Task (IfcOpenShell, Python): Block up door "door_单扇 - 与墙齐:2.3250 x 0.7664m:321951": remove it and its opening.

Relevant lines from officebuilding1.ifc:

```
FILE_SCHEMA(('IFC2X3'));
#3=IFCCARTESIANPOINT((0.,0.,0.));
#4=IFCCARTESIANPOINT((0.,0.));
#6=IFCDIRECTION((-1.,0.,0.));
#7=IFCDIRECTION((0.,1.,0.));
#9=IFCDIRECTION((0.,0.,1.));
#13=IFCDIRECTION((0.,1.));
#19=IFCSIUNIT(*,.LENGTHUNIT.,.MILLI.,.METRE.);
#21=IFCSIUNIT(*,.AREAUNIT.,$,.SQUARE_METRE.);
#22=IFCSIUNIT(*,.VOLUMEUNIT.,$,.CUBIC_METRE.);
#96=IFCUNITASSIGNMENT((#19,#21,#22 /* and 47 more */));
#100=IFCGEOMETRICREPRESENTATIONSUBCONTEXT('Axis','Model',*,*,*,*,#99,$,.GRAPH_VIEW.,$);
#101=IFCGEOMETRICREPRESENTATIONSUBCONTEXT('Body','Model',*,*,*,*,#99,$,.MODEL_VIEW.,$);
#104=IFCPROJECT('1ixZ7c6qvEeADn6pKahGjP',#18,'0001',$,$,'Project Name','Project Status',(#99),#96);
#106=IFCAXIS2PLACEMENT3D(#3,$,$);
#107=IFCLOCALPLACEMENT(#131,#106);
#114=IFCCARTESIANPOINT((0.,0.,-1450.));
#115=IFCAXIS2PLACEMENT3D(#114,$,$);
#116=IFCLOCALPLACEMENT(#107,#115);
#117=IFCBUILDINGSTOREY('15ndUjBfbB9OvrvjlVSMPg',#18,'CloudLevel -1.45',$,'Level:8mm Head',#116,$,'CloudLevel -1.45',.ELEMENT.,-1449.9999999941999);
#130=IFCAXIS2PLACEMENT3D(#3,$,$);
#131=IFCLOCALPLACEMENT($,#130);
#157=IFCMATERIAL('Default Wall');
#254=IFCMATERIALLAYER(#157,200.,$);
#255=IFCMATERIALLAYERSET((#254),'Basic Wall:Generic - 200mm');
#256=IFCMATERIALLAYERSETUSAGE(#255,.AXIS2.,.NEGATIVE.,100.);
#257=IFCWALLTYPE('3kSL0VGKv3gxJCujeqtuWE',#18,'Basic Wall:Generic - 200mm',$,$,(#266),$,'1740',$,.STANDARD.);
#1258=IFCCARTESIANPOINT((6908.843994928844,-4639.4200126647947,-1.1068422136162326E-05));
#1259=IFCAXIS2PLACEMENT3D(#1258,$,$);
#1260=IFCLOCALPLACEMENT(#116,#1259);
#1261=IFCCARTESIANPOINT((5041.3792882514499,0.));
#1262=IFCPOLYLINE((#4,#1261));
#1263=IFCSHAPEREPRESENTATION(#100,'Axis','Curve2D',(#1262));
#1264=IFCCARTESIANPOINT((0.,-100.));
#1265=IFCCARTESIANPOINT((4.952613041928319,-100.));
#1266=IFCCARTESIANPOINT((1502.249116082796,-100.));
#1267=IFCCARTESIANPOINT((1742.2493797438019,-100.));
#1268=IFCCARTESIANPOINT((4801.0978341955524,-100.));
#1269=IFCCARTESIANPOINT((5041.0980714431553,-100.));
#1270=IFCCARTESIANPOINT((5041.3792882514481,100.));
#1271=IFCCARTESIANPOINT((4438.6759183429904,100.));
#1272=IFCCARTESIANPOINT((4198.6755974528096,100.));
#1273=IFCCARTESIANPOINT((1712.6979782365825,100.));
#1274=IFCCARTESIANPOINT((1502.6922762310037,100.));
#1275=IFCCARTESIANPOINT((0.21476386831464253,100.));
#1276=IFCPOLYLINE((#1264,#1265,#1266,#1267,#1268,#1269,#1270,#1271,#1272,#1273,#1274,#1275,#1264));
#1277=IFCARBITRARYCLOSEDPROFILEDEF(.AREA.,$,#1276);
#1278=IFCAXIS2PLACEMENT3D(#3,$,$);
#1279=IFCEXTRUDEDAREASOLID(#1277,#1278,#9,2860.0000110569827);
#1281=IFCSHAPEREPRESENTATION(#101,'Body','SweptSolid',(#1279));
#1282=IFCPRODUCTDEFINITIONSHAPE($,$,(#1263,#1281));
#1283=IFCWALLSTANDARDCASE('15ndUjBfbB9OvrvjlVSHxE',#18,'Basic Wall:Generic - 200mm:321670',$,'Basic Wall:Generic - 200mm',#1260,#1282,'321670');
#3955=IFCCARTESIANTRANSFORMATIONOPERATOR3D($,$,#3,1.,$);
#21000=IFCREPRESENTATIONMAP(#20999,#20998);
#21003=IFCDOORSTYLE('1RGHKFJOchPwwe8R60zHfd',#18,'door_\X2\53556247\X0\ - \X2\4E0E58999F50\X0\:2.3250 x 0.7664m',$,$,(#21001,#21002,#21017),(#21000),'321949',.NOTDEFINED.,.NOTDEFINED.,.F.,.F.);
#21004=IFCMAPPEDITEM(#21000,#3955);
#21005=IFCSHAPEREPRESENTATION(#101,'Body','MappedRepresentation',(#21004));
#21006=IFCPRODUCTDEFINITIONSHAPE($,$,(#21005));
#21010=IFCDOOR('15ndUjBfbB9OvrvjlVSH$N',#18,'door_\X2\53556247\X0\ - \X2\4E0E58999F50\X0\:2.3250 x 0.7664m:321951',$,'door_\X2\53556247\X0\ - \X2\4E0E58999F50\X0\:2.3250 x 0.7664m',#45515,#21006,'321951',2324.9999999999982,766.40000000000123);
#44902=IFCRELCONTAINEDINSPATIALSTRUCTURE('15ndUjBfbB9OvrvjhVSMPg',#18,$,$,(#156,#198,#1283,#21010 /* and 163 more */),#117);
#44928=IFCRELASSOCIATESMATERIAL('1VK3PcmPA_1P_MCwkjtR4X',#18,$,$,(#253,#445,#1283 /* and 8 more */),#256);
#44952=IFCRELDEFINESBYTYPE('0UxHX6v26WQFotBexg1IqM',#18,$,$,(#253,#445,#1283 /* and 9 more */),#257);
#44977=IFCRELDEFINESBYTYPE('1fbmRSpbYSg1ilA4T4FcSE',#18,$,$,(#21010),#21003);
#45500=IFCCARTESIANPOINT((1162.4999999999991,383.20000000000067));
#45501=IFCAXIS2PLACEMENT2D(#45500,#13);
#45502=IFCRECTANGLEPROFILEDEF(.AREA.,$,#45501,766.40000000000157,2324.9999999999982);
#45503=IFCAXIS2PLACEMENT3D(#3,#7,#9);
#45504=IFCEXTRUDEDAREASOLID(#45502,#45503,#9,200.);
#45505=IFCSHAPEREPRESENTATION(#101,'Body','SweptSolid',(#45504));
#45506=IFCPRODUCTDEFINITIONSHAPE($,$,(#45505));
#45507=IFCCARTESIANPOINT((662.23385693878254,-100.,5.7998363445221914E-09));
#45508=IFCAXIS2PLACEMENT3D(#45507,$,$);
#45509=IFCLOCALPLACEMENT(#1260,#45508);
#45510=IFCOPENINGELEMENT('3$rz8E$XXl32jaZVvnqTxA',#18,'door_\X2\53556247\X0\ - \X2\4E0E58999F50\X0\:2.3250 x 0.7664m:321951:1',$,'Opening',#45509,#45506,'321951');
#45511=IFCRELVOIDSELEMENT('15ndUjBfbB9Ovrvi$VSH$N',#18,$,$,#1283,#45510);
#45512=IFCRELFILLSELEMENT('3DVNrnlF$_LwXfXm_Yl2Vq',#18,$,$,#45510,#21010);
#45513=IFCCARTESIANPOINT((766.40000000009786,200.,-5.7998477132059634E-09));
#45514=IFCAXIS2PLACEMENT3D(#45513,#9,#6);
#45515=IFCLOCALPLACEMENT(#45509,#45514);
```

```python
import ifcopenshell
import ifcopenshell.api.feature
import ifcopenshell.api.root
import ifcopenshell.geom
import ifcopenshell.util.shape

model = ifcopenshell.open("officebuilding1.ifc")
settings = ifcopenshell.geom.settings()


def volume(element):
    """Net volume in cubic metres, openings subtracted."""
    shape = ifcopenshell.geom.create_shape(settings, element)
    return ifcopenshell.util.shape.get_volume(shape.geometry)


door = model.by_guid("15ndUjBfbB9OvrvjlVSH$N")
opening = door.FillsVoids[0].RelatingOpeningElement
wall = opening.VoidsElements[0].RelatingBuildingElement
before = volume(wall)

ifcopenshell.api.root.remove_product(model, product=door)
ifcopenshell.api.feature.remove_feature(model, feature=opening)

after = volume(wall)

print(f"wall volume {before:.3f} -> {after:.3f} m3")

model.write("officebuilding1-out.ifc")
```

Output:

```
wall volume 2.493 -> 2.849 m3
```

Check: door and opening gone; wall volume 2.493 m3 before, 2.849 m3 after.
